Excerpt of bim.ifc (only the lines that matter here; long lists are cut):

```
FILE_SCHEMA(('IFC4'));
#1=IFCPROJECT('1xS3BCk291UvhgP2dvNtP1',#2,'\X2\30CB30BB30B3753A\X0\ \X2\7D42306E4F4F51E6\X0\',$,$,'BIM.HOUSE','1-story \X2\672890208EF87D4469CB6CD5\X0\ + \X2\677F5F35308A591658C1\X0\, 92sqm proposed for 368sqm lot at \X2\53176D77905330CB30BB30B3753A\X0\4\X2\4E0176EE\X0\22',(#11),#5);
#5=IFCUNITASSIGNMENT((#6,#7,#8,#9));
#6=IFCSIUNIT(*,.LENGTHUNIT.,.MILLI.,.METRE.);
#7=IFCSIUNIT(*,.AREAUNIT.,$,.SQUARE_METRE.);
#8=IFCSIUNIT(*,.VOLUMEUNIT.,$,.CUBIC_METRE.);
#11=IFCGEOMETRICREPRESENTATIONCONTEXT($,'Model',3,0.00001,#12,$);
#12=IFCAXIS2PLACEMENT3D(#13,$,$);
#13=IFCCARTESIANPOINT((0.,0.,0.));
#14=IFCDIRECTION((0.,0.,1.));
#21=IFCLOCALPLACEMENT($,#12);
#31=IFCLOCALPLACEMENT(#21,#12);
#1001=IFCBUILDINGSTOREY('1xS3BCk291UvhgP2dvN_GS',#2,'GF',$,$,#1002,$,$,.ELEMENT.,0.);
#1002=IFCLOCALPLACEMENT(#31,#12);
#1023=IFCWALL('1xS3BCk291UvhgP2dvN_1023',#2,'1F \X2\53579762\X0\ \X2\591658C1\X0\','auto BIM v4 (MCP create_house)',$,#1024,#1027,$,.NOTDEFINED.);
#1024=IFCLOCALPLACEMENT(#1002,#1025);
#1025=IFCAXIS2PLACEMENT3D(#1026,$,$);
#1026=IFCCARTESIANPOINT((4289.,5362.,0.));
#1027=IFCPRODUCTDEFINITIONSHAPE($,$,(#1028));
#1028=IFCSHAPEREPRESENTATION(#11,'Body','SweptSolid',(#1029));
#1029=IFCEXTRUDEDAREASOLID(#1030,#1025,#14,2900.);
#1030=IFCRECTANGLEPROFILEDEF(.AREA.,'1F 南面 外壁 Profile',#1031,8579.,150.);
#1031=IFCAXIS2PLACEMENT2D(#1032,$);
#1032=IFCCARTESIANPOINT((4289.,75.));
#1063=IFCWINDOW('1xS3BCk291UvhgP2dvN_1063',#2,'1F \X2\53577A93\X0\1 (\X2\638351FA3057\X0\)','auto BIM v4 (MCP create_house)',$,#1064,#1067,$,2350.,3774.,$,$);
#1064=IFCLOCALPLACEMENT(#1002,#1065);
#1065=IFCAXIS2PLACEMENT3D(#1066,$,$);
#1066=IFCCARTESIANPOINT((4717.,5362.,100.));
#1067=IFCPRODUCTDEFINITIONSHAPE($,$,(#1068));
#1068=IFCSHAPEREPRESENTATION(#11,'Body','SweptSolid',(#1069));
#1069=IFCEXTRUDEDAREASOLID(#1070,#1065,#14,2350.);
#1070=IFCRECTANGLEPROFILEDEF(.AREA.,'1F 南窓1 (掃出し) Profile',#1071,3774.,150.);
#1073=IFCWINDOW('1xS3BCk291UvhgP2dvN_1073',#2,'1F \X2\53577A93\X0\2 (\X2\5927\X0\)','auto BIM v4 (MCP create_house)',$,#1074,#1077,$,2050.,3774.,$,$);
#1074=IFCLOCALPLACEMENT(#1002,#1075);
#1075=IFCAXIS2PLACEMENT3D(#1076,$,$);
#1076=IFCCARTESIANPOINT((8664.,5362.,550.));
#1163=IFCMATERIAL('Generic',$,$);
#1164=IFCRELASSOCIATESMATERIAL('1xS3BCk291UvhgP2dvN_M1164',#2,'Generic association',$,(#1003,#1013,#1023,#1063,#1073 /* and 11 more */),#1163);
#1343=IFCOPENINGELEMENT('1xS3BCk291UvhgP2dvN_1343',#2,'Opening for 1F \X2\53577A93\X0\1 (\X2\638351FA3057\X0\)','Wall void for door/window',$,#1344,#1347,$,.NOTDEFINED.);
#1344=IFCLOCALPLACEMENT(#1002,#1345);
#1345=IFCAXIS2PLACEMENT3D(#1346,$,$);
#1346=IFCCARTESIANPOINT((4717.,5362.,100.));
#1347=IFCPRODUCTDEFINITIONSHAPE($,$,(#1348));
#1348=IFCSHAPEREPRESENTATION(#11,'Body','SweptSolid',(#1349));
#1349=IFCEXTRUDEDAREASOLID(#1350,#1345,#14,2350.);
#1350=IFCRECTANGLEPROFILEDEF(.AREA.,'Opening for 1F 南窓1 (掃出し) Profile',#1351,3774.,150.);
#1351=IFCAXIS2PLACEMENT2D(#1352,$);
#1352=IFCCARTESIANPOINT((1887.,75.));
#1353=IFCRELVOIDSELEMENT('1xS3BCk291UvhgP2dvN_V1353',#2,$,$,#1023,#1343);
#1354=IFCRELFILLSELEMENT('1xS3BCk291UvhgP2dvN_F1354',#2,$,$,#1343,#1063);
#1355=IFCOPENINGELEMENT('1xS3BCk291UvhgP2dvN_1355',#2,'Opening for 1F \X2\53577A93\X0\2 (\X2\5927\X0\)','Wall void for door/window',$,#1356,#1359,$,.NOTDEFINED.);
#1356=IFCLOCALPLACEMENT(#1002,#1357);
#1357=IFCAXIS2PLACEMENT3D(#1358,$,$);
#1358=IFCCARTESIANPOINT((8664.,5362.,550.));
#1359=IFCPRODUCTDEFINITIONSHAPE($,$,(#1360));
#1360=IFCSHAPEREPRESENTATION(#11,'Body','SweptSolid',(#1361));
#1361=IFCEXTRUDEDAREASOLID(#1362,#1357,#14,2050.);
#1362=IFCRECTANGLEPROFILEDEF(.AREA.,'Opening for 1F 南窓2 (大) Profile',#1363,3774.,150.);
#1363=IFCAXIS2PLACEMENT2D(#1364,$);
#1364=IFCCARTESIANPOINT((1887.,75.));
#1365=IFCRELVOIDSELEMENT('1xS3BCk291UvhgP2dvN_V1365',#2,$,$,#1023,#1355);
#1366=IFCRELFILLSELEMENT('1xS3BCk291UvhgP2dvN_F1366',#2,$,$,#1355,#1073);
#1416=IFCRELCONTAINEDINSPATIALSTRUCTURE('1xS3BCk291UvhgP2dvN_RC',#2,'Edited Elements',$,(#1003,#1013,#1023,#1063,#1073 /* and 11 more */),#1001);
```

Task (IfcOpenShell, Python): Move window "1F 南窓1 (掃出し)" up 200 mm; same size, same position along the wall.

```python
import numpy as np
import ifcopenshell
import ifcopenshell.api.geometry
import ifcopenshell.util.placement
import ifcopenshell.util.unit

model = ifcopenshell.open("bim.ifc")
unit_scale = ifcopenshell.util.unit.calculate_unit_scale(model)

window = model.by_guid("1xS3BCk291UvhgP2dvN_1063")
opening = window.FillsVoids[0].RelatingOpeningElement
dz = 0.2 / unit_scale

shift = np.array([0.0, 0.0, dz])
# The window is not placed relative to its opening, so move both.
for product in (opening, window):
    matrix = ifcopenshell.util.placement.get_local_placement(product.ObjectPlacement)
    matrix[:3, 3] += shift
    ifcopenshell.api.geometry.edit_object_placement(model, product=product, matrix=matrix, is_si=False)

print(f"moved by {dz * unit_scale:+.3f} m")

model.write("bim_edited.ifc")
```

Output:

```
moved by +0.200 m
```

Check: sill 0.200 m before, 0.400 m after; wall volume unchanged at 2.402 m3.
